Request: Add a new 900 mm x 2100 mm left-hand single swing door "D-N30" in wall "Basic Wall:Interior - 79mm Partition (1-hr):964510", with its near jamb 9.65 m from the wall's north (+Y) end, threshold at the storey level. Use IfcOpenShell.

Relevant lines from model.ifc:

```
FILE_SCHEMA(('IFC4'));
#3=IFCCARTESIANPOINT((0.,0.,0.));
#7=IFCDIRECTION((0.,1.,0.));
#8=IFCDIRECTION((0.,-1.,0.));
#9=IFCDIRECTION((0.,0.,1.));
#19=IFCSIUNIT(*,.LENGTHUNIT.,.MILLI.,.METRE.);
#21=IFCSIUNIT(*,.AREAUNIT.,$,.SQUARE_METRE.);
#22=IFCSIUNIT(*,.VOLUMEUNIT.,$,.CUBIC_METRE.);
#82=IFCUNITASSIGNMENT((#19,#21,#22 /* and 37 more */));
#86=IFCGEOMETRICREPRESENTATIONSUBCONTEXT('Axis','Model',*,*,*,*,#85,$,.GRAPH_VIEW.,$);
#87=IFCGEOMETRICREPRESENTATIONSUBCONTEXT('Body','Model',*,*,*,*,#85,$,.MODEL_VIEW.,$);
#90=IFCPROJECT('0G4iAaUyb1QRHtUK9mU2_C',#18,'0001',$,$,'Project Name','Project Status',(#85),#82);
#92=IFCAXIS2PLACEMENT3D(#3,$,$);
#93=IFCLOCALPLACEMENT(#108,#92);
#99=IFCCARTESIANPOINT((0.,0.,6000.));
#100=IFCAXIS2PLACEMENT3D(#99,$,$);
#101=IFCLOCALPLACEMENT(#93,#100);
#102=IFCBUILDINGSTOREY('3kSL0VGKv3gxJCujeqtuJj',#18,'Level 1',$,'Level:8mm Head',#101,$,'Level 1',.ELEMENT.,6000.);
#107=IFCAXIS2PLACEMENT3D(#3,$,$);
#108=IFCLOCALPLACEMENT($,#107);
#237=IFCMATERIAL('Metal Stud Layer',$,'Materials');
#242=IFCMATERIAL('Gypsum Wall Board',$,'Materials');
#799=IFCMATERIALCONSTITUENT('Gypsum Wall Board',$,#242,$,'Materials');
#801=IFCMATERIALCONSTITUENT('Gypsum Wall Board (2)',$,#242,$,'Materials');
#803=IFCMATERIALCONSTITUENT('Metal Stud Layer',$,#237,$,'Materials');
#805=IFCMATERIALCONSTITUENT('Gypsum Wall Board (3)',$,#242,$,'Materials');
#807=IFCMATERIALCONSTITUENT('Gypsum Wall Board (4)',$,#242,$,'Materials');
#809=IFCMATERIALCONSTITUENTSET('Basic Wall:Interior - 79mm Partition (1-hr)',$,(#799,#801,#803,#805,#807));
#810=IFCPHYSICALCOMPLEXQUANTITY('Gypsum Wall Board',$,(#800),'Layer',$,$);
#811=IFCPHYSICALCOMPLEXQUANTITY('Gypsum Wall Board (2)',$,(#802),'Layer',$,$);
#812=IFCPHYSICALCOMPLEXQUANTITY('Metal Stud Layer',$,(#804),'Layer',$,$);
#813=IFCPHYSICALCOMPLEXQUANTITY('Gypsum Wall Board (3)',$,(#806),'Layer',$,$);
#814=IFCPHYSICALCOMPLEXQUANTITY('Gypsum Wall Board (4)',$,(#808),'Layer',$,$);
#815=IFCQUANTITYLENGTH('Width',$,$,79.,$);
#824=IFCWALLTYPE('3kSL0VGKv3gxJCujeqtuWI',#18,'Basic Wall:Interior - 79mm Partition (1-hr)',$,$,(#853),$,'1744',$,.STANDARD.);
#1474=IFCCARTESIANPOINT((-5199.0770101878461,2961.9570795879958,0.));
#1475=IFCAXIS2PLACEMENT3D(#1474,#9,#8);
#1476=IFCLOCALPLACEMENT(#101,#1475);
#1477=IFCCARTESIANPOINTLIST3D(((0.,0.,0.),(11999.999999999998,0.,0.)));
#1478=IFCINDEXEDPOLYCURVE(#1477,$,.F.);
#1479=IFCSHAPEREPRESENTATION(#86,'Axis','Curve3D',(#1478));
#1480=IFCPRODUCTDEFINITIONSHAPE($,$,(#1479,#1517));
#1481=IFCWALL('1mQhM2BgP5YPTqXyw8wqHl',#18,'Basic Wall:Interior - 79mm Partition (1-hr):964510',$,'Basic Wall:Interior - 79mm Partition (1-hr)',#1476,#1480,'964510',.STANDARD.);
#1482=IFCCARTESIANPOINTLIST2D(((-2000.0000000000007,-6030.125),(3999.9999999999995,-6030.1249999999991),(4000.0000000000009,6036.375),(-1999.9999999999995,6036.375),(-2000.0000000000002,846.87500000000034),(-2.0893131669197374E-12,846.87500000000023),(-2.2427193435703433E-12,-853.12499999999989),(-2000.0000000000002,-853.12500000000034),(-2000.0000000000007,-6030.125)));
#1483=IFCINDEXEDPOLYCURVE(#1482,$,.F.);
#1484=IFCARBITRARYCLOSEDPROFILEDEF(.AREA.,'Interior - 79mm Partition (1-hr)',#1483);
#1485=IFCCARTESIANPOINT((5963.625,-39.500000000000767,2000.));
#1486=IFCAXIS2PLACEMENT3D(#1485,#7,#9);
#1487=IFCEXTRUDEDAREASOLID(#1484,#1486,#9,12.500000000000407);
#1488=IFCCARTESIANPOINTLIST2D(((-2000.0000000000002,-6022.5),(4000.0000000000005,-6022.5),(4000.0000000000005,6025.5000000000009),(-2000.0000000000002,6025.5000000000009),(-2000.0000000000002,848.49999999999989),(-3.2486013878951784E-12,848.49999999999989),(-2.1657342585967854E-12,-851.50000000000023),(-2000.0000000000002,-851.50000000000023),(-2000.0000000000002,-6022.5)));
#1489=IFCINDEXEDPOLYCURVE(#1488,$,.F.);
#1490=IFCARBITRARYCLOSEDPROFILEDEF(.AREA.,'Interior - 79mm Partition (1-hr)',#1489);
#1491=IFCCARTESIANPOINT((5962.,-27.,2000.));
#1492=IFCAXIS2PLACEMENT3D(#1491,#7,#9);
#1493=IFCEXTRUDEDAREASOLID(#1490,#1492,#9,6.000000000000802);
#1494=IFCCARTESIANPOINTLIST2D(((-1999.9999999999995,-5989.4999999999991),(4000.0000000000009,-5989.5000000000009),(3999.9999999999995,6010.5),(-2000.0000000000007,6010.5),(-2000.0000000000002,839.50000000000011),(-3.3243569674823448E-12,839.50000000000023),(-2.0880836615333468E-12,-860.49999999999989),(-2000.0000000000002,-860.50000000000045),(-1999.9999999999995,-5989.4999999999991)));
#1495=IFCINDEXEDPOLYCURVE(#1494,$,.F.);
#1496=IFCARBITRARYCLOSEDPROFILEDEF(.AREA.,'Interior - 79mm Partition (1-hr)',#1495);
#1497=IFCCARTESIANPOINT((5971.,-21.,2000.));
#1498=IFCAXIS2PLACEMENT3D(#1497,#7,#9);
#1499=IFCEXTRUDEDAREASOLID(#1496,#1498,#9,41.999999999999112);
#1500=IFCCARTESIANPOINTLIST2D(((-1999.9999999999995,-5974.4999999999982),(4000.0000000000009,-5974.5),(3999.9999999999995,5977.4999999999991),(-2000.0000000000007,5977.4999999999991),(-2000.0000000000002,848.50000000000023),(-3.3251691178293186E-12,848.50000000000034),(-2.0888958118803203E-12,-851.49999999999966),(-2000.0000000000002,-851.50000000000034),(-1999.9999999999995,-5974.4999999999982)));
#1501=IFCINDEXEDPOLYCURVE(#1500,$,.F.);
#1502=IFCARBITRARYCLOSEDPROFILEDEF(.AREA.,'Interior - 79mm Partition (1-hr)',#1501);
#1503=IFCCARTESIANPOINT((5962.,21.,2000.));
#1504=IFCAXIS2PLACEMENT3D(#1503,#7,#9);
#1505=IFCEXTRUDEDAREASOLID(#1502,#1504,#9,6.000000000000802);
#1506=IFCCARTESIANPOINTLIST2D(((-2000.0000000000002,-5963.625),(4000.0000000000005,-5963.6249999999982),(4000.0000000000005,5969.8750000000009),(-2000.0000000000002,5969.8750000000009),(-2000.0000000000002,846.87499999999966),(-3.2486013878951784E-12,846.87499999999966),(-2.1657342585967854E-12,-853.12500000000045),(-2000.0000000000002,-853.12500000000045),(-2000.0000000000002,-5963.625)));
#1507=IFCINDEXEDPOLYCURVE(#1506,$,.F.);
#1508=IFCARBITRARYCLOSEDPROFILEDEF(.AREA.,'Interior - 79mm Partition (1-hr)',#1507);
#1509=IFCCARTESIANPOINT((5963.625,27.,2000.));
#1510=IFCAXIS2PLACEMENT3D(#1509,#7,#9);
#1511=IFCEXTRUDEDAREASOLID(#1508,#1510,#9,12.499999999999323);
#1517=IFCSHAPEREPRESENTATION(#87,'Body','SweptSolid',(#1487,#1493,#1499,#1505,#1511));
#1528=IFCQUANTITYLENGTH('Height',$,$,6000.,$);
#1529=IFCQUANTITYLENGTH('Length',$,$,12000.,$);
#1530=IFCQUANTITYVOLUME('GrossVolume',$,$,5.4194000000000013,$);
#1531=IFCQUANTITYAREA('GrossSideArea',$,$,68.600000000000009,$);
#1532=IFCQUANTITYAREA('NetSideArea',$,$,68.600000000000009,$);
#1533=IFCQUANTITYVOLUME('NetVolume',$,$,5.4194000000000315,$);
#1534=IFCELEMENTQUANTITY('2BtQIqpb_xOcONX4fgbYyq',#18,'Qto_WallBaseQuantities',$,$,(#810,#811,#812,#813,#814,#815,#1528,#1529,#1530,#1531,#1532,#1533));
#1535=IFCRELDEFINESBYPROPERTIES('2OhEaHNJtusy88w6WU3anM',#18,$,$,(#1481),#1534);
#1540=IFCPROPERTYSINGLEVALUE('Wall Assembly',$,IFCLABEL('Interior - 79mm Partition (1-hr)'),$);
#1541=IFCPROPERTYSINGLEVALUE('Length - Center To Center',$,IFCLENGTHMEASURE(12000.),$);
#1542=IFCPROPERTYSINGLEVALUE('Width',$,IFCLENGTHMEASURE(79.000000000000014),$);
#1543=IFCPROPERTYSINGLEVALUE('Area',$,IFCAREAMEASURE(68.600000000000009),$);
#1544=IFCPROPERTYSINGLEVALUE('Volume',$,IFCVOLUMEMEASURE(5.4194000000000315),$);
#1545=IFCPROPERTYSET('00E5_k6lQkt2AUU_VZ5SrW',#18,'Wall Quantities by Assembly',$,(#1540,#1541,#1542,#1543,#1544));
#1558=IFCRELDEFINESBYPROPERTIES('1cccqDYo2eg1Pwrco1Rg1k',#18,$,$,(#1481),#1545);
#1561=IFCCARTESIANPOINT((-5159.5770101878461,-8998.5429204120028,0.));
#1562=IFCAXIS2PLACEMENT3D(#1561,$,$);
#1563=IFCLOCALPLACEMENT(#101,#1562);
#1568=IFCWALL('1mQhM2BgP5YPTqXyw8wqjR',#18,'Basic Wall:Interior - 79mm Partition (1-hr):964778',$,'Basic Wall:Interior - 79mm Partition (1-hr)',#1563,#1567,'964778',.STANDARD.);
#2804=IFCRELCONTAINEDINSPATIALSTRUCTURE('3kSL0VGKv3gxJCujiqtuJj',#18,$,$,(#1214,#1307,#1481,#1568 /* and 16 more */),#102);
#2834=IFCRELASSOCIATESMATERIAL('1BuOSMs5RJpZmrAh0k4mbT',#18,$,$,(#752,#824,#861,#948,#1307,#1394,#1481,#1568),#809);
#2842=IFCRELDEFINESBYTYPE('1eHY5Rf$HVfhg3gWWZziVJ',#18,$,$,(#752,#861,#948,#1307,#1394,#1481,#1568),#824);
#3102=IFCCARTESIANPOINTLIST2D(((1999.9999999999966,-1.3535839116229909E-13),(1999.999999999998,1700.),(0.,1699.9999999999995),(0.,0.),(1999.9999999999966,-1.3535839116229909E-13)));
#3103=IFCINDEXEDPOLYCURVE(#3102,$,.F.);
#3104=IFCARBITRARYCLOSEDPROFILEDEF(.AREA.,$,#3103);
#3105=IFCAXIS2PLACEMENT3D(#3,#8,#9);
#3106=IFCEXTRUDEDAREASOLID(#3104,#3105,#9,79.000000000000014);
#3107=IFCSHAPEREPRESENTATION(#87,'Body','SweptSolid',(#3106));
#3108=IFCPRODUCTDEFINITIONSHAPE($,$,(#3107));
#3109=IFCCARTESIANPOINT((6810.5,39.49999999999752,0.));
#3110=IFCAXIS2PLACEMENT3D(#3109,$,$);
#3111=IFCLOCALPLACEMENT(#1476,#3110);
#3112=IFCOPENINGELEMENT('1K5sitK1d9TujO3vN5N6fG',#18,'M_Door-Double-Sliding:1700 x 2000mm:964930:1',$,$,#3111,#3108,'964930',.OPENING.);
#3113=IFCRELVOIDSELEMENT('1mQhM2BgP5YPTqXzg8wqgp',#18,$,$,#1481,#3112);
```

```python
import numpy as np
import ifcopenshell
import ifcopenshell.api.feature
import ifcopenshell.api.geometry
import ifcopenshell.api.pset
import ifcopenshell.api.root
import ifcopenshell.api.spatial
import ifcopenshell.geom
import ifcopenshell.util.element
import ifcopenshell.util.placement
import ifcopenshell.util.representation
import ifcopenshell.util.shape
import ifcopenshell.util.unit

model = ifcopenshell.open("model.ifc")
unit_scale = ifcopenshell.util.unit.calculate_unit_scale(model)
area_scale = ifcopenshell.util.unit.calculate_unit_scale(model, "AREAUNIT")
volume_scale = ifcopenshell.util.unit.calculate_unit_scale(model, "VOLUMEUNIT")
settings = ifcopenshell.geom.settings()


def volume(element):
    """Net volume in cubic metres, openings subtracted."""
    shape = ifcopenshell.geom.create_shape(settings, element)
    return ifcopenshell.util.shape.get_volume(shape.geometry)


wall = model.by_guid("1mQhM2BgP5YPTqXyw8wqHl")
storey = ifcopenshell.util.element.get_container(wall, ifc_class="IfcBuildingStorey")
context = ifcopenshell.util.representation.get_context(model, "Model", "Body", "MODEL_VIEW")
before = volume(wall)

width, height, from_end, sill = 0.9, 2.1, 9.65, 0.0  # metres

# The wall runs along its own X axis, and the end named is its -X end.
wall_shape = ifcopenshell.geom.create_shape(settings, wall)
x, y, z = ifcopenshell.util.shape.get_vertices(wall_shape.geometry).T
start = x.min() + from_end
face, thickness = float(y.min()), float(y.max() - y.min())
wall_matrix = ifcopenshell.util.placement.get_local_placement(wall.ObjectPlacement)
level = ifcopenshell.util.placement.get_local_placement(storey.ObjectPlacement)[2, 3]


def in_wall(x, y):
    """Placement at x, y metres in the wall's axes, at sill height."""
    matrix = wall_matrix.copy()
    matrix[:, 3] = wall_matrix @ np.array([x / unit_scale, y / unit_scale, 0.0, 1.0])
    matrix[2, 3] = level + sill / unit_scale
    return matrix


# Opening: a box that overshoots both wall faces by 50 mm.
opening = ifcopenshell.api.root.create_entity(model, ifc_class="IfcOpeningElement", predefined_type="OPENING")
box = ifcopenshell.api.geometry.add_wall_representation(
    model, context=context, length=width, height=height, thickness=thickness + 0.1
)
ifcopenshell.api.geometry.assign_representation(model, product=opening, representation=box)
ifcopenshell.api.geometry.edit_object_placement(model, product=opening, matrix=in_wall(start, face - 0.05), is_si=False)
ifcopenshell.api.feature.add_feature(model, feature=opening, element=wall)

door = ifcopenshell.api.root.create_entity(model, ifc_class="IfcDoor", name="D-N30", predefined_type="DOOR")
door.OverallWidth, door.OverallHeight = width / unit_scale, height / unit_scale
door.OperationType = "SINGLE_SWING_LEFT"
body = ifcopenshell.api.geometry.add_door_representation(
    model,
    context=context,
    overall_width=door.OverallWidth,
    overall_height=door.OverallHeight,
    operation_type="SINGLE_SWING_LEFT",
    lining_properties={"LiningDepth": thickness / unit_scale, "ThresholdDepth": thickness / unit_scale},
)
ifcopenshell.api.geometry.assign_representation(model, product=door, representation=body)
ifcopenshell.api.spatial.assign_container(model, products=[door], relating_structure=storey)
ifcopenshell.api.feature.add_filling(model, opening=opening, element=door)

# The lining spans the wall, so the door starts at the wall face.
ifcopenshell.api.geometry.edit_object_placement(model, product=door, matrix=in_wall(start, face), is_si=False)

after = volume(wall)

# Update the wall's stored quantities.
qto = model.by_id(ifcopenshell.util.element.get_pset(wall, "Qto_WallBaseQuantities", should_inherit=False)["id"])
ifcopenshell.api.pset.edit_qto(model, qto=qto, properties={
    "NetSideArea": after / thickness / area_scale,
    "NetVolume": after / volume_scale,
})
pset = model.by_id(ifcopenshell.util.element.get_pset(wall, "Wall Quantities by Assembly", should_inherit=False)["id"])
ifcopenshell.api.pset.edit_pset(model, pset=pset, properties={
    "Area": model.create_entity("IfcAreaMeasure", after / thickness / area_scale),
    "Volume": model.create_entity("IfcVolumeMeasure", after / volume_scale),
})

print(f"wall volume {before:.3f} -> {after:.3f} m3")

model.write("model_edited.ifc")
```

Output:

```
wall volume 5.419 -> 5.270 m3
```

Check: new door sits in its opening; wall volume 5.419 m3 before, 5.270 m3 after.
